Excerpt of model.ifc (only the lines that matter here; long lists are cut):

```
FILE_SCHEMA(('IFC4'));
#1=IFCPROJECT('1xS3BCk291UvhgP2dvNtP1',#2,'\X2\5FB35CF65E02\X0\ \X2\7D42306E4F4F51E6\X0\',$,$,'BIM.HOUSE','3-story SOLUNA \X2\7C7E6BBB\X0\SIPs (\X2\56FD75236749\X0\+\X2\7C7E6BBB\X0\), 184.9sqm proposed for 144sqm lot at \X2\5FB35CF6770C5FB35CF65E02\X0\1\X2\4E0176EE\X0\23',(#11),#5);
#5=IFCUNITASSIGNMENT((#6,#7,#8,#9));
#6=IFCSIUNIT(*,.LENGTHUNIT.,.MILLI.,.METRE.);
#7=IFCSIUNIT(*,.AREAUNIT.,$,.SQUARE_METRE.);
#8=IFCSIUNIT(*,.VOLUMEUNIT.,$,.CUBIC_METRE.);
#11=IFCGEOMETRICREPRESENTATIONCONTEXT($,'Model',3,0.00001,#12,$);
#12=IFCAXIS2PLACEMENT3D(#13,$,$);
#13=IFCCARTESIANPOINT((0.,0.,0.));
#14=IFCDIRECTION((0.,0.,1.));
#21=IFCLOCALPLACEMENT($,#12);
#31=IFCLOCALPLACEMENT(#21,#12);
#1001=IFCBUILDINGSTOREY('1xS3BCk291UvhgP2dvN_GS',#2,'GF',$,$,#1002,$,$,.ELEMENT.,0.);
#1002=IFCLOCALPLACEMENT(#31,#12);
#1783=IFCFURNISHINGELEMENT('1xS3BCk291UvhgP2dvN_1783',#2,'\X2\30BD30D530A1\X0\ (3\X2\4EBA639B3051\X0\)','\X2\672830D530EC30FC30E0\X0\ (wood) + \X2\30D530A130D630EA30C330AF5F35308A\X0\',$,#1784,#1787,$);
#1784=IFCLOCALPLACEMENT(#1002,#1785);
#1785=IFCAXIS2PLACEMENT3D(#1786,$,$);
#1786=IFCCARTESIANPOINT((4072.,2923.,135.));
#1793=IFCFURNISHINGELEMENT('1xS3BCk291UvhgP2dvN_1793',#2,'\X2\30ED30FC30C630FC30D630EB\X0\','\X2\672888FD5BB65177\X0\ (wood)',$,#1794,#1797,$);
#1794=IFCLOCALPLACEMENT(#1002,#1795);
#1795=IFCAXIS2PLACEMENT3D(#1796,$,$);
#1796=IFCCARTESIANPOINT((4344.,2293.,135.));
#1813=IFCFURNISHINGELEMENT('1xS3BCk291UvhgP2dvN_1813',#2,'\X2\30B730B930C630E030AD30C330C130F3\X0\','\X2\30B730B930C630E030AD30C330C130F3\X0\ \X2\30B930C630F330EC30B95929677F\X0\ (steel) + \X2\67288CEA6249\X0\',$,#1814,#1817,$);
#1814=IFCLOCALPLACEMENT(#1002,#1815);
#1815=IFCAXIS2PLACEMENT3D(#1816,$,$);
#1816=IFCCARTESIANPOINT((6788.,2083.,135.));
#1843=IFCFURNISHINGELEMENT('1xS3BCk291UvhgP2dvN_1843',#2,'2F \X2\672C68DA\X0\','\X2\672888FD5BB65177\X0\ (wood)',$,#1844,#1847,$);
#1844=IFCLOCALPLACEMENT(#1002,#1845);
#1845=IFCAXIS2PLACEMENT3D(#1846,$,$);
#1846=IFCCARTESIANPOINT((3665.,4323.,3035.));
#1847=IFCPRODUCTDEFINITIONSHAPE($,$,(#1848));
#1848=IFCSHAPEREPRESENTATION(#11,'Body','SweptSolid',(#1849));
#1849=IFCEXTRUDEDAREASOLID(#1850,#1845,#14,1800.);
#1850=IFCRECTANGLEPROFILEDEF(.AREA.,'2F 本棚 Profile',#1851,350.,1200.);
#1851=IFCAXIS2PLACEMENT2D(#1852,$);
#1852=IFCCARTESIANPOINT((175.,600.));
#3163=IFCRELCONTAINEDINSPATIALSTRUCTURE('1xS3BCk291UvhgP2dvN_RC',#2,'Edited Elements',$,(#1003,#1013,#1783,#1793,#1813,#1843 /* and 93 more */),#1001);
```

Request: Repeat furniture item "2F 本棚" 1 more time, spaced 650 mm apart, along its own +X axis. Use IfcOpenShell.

```python
import ifcopenshell
import ifcopenshell.api.geometry
import ifcopenshell.api.root
import ifcopenshell.util.element
import ifcopenshell.util.placement
import ifcopenshell.util.unit

model = ifcopenshell.open("model.ifc")
unit_scale = ifcopenshell.util.unit.calculate_unit_scale(model)


def reuse_history(source, copy):
    """copy_class also copies each property set's owner history, people and application; keep the originals."""
    for rel in copy.IsDefinedBy:
        if rel.is_a("IfcRelDefinesByProperties") and (history := rel.RelatingPropertyDefinition.OwnerHistory):
            rel.RelatingPropertyDefinition.OwnerHistory = source.OwnerHistory
            ifcopenshell.util.element.remove_deep2(model, history)


source = model.by_guid("1xS3BCk291UvhgP2dvN_1843")
base = ifcopenshell.util.placement.get_local_placement(source.ObjectPlacement)
step = base[:3, 0] * 0.65 / unit_scale

for i in range(1, 2):
    copy = ifcopenshell.api.root.copy_class(model, product=source)
    copy.Representation = ifcopenshell.util.element.copy_deep(
        model, source.Representation, exclude=["IfcGeometricRepresentationContext", "IfcRepresentationMap"]
    )
    reuse_history(source, copy)
    matrix = base.copy()
    matrix[:3, 3] += i * step
    print("added at", matrix[:3, 3].round(3) + 0.0)
    ifcopenshell.api.geometry.edit_object_placement(model, product=copy, matrix=matrix, is_si=False)

model.write("model-out.ifc")
```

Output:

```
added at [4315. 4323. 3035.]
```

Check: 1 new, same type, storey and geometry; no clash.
